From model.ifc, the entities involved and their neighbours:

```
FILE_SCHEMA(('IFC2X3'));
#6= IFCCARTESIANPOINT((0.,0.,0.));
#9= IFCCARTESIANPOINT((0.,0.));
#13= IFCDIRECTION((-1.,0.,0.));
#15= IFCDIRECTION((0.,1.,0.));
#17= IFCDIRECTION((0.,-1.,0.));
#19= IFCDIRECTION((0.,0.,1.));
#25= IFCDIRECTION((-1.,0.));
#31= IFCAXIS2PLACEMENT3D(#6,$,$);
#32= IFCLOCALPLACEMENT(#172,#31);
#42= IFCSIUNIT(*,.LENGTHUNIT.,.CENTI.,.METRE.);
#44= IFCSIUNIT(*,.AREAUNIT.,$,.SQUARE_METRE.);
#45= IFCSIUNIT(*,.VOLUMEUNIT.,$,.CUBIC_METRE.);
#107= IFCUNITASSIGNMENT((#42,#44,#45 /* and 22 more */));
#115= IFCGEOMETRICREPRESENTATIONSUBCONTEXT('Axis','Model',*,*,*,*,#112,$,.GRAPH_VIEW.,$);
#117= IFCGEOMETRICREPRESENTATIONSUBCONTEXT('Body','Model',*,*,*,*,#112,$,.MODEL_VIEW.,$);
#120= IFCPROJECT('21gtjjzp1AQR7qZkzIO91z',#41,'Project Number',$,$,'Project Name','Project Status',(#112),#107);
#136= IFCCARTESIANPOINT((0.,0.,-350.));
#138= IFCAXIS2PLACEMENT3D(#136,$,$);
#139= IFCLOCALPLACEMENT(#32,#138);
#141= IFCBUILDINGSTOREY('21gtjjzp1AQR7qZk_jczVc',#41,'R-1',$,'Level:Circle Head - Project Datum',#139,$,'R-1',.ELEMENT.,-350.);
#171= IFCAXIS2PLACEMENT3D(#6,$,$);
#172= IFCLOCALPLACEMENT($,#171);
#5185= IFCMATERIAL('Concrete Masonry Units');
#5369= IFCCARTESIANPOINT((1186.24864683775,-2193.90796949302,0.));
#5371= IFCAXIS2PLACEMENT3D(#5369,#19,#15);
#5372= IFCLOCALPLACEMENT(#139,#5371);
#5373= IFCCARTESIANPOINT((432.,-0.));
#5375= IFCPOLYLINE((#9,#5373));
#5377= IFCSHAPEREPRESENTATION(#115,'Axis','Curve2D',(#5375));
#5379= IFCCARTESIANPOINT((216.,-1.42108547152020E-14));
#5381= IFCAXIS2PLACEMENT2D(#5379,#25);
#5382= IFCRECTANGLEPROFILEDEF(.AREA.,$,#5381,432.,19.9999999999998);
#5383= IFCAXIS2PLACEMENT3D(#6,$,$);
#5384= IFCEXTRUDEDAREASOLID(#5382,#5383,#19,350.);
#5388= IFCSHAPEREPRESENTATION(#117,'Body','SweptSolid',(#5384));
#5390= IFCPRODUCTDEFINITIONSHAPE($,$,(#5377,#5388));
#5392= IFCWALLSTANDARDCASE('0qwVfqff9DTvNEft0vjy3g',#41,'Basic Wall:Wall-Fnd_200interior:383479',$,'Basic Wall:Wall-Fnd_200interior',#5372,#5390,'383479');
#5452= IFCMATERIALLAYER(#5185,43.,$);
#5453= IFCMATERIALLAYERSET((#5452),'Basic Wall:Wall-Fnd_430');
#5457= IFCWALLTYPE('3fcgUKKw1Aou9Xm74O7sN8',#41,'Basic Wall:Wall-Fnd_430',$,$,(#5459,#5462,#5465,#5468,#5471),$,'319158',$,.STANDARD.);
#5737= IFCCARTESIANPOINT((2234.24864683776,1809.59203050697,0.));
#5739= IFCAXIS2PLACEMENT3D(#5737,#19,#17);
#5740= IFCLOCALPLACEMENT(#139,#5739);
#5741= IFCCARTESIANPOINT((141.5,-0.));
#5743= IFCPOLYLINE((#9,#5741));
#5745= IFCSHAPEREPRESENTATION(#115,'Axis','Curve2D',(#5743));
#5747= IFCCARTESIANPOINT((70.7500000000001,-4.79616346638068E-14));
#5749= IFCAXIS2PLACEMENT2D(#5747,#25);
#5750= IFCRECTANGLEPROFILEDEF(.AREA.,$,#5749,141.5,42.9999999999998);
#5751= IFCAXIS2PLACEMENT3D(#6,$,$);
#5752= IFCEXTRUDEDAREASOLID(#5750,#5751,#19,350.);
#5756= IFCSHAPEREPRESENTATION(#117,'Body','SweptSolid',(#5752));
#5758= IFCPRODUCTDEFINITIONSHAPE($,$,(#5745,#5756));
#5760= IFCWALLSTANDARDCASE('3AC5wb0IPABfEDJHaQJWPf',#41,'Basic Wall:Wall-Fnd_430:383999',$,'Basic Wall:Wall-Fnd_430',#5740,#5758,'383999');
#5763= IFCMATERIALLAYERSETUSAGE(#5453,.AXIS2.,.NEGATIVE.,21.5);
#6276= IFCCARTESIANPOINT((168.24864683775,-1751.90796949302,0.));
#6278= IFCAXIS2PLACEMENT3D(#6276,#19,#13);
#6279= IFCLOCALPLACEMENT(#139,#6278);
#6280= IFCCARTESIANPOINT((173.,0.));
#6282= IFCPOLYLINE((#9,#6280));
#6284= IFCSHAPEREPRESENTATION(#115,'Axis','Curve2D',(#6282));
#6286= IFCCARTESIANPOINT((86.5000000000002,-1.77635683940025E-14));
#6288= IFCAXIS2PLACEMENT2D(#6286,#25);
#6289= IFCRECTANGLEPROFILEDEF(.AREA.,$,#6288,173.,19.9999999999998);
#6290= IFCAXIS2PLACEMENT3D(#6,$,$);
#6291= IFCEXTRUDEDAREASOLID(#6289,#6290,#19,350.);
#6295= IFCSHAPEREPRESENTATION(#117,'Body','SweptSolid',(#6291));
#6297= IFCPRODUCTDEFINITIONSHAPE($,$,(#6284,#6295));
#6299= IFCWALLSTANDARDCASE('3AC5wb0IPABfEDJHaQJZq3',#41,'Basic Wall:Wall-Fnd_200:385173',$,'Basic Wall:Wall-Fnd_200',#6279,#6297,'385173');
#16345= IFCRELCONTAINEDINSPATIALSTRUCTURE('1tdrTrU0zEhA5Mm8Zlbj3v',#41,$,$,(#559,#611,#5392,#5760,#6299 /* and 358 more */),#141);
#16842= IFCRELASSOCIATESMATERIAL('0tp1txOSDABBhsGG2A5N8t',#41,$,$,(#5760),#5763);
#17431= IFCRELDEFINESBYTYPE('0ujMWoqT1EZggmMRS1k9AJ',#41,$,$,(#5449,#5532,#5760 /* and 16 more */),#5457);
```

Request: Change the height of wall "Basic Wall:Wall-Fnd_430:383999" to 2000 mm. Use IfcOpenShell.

```python
import ifcopenshell
import ifcopenshell.geom
import ifcopenshell.util.representation
import ifcopenshell.util.shape
import ifcopenshell.util.unit

model = ifcopenshell.open("model.ifc")
unit_scale = ifcopenshell.util.unit.calculate_unit_scale(model)
settings = ifcopenshell.geom.settings()


def volume(element):
    """Net volume in cubic metres, openings subtracted."""
    shape = ifcopenshell.geom.create_shape(settings, element)
    return ifcopenshell.util.shape.get_volume(shape.geometry)


wall = model.by_guid("3AC5wb0IPABfEDJHaQJWPf")
before = volume(wall)

body = ifcopenshell.util.representation.get_representation(wall, "Model", "Body")
solid = body.Items[0]
old_height = solid.Depth
solid.Depth = 2 / unit_scale
after = volume(wall)

print(f"height {old_height:g} -> {solid.Depth:g}, volume {before:.3f} -> {after:.3f} m3")

model.write("model_rev.ifc")
```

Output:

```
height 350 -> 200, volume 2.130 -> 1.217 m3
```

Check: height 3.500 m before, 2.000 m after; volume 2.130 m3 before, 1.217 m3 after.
